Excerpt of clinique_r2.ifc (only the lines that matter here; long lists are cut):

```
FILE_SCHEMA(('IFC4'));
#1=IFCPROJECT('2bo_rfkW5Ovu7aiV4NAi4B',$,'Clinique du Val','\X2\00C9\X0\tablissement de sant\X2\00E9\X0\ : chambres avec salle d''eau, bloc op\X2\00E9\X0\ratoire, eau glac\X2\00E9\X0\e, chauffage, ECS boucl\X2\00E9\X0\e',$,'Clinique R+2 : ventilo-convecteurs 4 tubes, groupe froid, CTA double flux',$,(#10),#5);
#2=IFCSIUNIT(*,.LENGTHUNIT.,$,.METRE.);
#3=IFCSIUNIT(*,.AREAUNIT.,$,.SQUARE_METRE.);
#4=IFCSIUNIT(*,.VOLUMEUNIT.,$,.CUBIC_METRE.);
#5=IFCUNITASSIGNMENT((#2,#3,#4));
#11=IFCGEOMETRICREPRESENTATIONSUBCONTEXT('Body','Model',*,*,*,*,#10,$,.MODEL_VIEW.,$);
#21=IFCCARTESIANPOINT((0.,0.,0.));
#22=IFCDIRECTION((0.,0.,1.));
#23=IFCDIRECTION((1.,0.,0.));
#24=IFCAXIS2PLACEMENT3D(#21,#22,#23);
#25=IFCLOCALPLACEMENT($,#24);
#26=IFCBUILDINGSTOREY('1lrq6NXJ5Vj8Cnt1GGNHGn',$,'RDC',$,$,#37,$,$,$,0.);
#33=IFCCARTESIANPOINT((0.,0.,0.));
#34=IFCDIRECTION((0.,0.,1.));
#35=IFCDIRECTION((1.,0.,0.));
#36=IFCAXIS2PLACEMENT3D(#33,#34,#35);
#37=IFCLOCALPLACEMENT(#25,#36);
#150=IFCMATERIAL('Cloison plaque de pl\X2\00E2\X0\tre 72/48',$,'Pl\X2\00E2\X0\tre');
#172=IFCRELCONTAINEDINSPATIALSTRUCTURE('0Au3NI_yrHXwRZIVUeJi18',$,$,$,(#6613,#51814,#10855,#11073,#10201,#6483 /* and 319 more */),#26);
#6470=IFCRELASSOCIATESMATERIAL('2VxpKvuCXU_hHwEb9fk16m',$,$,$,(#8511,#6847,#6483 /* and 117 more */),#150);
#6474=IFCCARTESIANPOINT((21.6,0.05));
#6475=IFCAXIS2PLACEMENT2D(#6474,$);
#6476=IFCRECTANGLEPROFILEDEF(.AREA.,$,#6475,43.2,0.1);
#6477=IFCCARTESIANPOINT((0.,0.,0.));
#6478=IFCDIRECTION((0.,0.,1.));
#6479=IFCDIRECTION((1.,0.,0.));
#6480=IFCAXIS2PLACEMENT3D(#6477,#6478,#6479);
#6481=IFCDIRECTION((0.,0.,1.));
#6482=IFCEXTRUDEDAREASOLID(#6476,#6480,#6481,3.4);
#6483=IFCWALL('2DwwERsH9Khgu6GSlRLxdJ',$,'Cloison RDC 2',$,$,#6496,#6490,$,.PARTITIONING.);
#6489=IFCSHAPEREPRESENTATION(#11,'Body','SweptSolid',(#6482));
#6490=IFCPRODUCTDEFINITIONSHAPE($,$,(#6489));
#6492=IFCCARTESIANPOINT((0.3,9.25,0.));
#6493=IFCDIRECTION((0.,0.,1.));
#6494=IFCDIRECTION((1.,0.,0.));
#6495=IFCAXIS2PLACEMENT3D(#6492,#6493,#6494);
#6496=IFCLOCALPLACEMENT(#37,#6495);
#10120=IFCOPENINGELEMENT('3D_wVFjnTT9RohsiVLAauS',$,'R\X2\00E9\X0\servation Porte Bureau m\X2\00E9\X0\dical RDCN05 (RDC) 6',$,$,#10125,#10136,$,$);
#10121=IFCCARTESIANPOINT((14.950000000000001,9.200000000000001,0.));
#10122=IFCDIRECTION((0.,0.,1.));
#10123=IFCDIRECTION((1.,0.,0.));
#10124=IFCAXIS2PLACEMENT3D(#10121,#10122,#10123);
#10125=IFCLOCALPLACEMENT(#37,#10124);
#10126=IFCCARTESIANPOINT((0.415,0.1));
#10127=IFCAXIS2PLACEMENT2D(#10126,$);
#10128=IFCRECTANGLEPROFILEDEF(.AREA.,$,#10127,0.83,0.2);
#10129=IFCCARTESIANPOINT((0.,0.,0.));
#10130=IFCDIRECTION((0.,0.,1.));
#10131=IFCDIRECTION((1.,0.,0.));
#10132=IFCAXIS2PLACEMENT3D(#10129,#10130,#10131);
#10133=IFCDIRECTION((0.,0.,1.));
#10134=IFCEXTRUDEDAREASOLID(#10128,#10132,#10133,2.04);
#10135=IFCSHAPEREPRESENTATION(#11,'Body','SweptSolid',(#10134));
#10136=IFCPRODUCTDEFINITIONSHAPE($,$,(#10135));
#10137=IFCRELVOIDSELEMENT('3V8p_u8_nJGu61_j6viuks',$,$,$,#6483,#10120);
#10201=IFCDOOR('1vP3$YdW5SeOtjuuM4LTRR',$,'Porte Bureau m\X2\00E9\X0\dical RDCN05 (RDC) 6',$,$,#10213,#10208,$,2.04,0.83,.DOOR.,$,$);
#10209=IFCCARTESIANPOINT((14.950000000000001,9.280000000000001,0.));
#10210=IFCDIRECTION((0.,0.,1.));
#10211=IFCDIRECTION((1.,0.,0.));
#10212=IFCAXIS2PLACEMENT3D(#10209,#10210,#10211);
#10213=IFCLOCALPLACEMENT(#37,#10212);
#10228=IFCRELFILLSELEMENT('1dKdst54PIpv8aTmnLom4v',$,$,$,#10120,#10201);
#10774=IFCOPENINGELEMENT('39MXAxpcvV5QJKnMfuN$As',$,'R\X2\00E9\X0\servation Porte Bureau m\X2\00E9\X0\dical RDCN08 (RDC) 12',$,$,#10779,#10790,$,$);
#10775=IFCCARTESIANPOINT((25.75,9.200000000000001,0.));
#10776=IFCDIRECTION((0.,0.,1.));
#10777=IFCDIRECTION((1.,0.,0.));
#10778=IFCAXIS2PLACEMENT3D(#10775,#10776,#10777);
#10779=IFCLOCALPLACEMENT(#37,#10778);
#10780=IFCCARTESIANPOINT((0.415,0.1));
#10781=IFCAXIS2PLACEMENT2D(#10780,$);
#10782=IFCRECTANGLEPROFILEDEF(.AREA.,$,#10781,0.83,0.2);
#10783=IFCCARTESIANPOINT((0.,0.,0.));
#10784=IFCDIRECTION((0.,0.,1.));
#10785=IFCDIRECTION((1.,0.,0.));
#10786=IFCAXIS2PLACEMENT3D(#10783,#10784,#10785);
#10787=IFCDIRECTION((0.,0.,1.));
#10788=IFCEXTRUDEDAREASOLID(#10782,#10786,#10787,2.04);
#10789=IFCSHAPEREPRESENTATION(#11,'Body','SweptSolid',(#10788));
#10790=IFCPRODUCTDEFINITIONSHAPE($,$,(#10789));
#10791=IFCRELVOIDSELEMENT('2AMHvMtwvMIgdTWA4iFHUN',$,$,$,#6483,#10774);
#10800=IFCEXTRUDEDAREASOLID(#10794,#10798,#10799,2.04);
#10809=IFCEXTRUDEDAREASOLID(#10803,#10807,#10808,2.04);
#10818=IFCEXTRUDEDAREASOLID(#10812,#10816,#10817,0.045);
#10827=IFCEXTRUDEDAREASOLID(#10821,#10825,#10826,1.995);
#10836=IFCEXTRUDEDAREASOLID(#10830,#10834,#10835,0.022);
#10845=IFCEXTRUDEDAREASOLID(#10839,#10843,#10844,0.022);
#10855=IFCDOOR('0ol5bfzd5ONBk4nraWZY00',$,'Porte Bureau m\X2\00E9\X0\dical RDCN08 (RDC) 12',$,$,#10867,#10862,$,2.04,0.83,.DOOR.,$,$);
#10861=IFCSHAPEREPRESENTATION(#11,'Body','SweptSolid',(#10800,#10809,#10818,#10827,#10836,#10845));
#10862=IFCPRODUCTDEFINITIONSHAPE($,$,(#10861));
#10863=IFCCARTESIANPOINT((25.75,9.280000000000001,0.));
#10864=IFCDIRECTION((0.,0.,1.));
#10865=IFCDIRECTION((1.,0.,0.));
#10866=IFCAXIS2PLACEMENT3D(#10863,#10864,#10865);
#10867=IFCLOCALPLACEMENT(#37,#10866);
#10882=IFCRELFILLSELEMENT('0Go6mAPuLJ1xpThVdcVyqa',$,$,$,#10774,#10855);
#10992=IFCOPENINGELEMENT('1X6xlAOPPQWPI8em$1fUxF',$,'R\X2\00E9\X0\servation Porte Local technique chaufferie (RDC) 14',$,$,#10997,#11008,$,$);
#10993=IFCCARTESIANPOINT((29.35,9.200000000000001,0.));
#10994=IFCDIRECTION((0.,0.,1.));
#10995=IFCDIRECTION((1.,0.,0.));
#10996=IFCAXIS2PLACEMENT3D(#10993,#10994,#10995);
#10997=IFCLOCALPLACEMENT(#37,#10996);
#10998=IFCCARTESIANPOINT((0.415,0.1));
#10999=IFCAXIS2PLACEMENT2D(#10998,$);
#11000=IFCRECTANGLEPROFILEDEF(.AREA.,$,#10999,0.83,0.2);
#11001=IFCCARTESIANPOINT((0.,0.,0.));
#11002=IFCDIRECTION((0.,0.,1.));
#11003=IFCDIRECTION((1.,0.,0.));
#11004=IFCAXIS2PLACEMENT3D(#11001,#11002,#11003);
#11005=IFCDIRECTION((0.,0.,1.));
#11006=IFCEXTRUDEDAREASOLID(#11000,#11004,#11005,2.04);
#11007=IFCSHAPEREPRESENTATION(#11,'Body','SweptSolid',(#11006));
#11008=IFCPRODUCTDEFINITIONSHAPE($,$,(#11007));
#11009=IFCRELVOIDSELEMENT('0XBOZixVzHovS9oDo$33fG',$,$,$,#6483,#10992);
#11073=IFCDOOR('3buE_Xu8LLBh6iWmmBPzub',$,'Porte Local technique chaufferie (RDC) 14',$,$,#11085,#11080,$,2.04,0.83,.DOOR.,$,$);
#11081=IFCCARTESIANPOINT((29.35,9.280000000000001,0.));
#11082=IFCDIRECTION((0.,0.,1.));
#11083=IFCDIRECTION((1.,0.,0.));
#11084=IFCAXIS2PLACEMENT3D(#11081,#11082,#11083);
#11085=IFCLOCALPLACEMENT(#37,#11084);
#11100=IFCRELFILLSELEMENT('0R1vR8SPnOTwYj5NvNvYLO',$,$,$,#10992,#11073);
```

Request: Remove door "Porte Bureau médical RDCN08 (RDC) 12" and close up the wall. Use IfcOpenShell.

```python
import ifcopenshell
import ifcopenshell.api.feature
import ifcopenshell.api.root
import ifcopenshell.geom
import ifcopenshell.util.shape

model = ifcopenshell.open("clinique_r2.ifc")
settings = ifcopenshell.geom.settings()


def volume(element):
    """Net volume in cubic metres, openings subtracted."""
    shape = ifcopenshell.geom.create_shape(settings, element)
    return ifcopenshell.util.shape.get_volume(shape.geometry)


door = model.by_guid("0ol5bfzd5ONBk4nraWZY00")
opening = door.FillsVoids[0].RelatingOpeningElement
wall = opening.VoidsElements[0].RelatingBuildingElement
before = volume(wall)

ifcopenshell.api.root.remove_product(model, product=door)
ifcopenshell.api.feature.remove_feature(model, feature=opening)

after = volume(wall)

print(f"wall volume {before:.3f} -> {after:.3f} m3")

model.write("clinique_r2_updated.ifc")
```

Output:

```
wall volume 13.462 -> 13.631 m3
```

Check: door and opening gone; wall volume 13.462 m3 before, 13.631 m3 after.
